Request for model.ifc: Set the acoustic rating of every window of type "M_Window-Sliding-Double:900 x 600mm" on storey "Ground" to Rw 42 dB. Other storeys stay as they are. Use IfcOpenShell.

First a look at what the model holds.

```python
import ifcopenshell
import ifcopenshell.util.element

model = ifcopenshell.open("model.ifc")
print(model.schema)
storey = next(s for s in model.by_type("IfcBuildingStorey") if s.Name == "Ground")
windows = [e for e in ifcopenshell.util.element.get_decomposition(storey) if e.is_a("IfcWindow")]
seen = {}
for e in windows:
    element_type = ifcopenshell.util.element.get_type(e)
    key = (element_type.Name if element_type != e and element_type else None, ifcopenshell.util.element.get_pset(e, "Pset_WindowCommon", "AcousticRating"))
    seen[key] = seen.get(key, 0) + 1
for (name, value), count in sorted(seen.items(), key=str):
    print(count, "x", name, "|", value)
```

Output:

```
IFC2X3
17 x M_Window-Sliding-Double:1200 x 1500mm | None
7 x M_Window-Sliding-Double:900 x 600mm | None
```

```python
import ifcopenshell
import ifcopenshell.api.pset
import ifcopenshell.util.element

model = ifcopenshell.open("model.ifc")

storey = next(s for s in model.by_type("IfcBuildingStorey") if s.Name == "Ground")
windows = [e for e in ifcopenshell.util.element.get_decomposition(storey) if e.is_a("IfcWindow")]

count = 0
for e in windows:
    element_type = ifcopenshell.util.element.get_type(e)
    if element_type in (None, e) or element_type.Name != "M_Window-Sliding-Double:900 x 600mm":
        continue
    # add_pset returns the element's existing set when there is one.
    pset = ifcopenshell.api.pset.add_pset(model, product=e, name="Pset_WindowCommon")
    ifcopenshell.api.pset.edit_pset(model, pset=pset, properties={"AcousticRating": "Rw 42 dB"})
    count += 1

print(count, "windows updated")

model.write("model_v2.ifc")
```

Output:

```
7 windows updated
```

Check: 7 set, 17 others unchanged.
